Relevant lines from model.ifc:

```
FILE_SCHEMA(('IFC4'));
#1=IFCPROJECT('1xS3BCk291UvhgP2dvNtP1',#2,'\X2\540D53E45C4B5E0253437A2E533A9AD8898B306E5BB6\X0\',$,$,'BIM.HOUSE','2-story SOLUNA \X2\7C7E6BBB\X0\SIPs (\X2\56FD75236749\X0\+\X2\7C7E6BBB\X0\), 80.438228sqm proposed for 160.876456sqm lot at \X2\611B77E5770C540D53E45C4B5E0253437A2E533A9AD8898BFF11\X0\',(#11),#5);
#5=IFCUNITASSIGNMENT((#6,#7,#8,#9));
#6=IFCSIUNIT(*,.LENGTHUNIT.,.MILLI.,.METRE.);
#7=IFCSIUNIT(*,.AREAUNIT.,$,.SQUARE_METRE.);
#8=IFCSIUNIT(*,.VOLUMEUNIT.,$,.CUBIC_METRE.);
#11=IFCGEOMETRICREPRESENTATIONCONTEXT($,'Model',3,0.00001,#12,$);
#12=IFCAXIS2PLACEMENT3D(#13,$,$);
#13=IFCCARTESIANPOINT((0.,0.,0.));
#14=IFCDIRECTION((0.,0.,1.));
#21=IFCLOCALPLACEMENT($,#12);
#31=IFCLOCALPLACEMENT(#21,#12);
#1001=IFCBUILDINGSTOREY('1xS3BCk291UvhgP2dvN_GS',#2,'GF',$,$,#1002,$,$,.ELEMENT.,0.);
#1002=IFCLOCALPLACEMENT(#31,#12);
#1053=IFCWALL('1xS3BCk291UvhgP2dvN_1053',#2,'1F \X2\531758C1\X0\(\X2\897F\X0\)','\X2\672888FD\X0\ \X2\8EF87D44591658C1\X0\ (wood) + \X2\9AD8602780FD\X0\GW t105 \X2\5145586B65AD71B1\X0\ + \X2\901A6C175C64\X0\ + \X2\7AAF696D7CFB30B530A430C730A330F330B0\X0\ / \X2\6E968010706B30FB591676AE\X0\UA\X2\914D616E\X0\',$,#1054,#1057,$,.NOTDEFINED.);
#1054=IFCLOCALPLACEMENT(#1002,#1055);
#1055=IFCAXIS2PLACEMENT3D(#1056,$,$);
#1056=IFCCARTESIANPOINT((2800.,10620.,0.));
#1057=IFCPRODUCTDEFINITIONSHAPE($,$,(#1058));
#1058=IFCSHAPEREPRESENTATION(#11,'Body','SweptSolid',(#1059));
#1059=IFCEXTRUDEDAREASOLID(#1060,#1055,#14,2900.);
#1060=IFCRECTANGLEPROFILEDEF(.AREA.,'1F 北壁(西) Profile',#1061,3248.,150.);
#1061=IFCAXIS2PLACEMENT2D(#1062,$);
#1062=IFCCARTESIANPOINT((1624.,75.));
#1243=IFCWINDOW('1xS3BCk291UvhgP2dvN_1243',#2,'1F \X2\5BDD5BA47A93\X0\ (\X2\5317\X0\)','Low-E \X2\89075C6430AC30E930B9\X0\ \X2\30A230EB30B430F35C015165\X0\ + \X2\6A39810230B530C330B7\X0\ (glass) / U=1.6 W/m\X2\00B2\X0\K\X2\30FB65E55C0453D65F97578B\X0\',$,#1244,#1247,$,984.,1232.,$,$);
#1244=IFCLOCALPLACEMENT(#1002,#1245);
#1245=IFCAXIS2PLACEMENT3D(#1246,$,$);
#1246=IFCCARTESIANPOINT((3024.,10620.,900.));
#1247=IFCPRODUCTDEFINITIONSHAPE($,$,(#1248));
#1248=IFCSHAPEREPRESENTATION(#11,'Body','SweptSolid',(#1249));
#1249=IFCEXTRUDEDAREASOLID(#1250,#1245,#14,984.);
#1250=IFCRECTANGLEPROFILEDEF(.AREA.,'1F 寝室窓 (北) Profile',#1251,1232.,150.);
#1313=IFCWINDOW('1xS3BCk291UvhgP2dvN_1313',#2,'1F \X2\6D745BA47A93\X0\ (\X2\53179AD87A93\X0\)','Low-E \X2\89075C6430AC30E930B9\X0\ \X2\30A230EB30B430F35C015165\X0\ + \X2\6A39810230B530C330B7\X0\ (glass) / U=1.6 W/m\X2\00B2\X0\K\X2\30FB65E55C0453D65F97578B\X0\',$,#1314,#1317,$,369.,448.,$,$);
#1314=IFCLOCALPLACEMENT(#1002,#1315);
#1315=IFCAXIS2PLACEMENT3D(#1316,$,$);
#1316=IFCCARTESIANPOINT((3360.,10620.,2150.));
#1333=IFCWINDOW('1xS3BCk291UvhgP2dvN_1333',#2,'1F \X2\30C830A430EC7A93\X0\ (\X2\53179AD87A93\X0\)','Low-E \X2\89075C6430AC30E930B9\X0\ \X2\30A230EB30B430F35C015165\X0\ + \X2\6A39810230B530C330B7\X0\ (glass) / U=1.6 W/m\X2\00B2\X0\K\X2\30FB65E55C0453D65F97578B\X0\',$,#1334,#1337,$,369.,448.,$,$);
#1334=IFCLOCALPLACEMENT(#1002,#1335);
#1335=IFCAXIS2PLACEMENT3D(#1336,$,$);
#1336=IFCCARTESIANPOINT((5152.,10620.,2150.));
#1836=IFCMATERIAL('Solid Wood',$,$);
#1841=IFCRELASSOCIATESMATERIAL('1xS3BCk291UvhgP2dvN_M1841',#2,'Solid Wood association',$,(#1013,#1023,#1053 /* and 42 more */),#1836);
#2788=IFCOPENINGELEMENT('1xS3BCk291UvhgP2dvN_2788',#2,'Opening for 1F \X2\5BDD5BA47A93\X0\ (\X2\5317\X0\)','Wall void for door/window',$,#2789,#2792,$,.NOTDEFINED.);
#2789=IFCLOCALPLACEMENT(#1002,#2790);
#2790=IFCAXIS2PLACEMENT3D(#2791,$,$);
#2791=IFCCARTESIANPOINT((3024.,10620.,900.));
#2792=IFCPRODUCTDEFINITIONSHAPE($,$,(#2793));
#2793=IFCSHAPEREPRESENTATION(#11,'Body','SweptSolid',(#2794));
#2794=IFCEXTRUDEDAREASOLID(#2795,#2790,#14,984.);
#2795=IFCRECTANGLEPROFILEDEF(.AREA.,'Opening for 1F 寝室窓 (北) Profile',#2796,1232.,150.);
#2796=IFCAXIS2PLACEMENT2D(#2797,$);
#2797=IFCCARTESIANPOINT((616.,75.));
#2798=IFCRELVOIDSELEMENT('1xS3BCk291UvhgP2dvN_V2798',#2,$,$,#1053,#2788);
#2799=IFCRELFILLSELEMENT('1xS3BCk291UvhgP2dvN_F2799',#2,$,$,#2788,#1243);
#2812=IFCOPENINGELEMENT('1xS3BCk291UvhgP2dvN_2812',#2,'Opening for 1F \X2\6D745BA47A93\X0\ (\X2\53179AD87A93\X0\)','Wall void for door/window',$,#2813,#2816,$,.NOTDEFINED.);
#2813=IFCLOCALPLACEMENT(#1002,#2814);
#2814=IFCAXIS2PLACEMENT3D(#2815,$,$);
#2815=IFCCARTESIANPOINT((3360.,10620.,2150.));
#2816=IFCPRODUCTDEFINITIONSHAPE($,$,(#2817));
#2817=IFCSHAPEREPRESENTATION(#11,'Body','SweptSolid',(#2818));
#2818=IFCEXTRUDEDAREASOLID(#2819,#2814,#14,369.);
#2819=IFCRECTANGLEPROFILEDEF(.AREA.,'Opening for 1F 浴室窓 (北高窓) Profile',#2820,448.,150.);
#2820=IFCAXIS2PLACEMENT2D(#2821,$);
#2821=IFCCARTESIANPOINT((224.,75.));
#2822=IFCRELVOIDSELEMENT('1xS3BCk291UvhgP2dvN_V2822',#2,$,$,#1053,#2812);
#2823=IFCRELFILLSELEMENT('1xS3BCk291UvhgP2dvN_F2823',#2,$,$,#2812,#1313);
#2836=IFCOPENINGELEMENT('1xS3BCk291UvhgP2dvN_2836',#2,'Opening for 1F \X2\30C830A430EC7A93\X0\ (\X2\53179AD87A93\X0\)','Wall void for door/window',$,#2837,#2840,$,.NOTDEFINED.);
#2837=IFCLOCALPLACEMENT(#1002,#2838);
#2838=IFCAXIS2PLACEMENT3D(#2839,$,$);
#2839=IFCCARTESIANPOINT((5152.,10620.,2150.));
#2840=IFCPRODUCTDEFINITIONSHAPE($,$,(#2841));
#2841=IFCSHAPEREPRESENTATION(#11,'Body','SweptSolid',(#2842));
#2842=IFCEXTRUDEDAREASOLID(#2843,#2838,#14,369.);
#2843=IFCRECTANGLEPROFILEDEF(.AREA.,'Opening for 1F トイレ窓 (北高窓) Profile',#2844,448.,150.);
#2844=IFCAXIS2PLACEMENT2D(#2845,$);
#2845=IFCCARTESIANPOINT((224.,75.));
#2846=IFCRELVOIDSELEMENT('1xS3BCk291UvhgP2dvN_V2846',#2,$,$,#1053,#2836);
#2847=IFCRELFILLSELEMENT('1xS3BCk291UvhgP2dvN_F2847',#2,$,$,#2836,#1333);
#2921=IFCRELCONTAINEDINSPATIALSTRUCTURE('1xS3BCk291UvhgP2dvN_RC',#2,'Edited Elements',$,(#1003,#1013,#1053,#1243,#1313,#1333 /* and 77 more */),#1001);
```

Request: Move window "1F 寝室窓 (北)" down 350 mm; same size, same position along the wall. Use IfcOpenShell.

```python
import numpy as np
import ifcopenshell
import ifcopenshell.api.geometry
import ifcopenshell.util.placement
import ifcopenshell.util.unit

model = ifcopenshell.open("model.ifc")
unit_scale = ifcopenshell.util.unit.calculate_unit_scale(model)

window = model.by_guid("1xS3BCk291UvhgP2dvN_1243")
opening = window.FillsVoids[0].RelatingOpeningElement
dz = -0.35 / unit_scale

shift = np.array([0.0, 0.0, dz])
# The window is not placed relative to its opening, so move both.
for product in (opening, window):
    matrix = ifcopenshell.util.placement.get_local_placement(product.ObjectPlacement)
    matrix[:3, 3] += shift
    ifcopenshell.api.geometry.edit_object_placement(model, product=product, matrix=matrix, is_si=False)

print(f"moved by {dz * unit_scale:+.3f} m")

model.write("model_v2.ifc")
```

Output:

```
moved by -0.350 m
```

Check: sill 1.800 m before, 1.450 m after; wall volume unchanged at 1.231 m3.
